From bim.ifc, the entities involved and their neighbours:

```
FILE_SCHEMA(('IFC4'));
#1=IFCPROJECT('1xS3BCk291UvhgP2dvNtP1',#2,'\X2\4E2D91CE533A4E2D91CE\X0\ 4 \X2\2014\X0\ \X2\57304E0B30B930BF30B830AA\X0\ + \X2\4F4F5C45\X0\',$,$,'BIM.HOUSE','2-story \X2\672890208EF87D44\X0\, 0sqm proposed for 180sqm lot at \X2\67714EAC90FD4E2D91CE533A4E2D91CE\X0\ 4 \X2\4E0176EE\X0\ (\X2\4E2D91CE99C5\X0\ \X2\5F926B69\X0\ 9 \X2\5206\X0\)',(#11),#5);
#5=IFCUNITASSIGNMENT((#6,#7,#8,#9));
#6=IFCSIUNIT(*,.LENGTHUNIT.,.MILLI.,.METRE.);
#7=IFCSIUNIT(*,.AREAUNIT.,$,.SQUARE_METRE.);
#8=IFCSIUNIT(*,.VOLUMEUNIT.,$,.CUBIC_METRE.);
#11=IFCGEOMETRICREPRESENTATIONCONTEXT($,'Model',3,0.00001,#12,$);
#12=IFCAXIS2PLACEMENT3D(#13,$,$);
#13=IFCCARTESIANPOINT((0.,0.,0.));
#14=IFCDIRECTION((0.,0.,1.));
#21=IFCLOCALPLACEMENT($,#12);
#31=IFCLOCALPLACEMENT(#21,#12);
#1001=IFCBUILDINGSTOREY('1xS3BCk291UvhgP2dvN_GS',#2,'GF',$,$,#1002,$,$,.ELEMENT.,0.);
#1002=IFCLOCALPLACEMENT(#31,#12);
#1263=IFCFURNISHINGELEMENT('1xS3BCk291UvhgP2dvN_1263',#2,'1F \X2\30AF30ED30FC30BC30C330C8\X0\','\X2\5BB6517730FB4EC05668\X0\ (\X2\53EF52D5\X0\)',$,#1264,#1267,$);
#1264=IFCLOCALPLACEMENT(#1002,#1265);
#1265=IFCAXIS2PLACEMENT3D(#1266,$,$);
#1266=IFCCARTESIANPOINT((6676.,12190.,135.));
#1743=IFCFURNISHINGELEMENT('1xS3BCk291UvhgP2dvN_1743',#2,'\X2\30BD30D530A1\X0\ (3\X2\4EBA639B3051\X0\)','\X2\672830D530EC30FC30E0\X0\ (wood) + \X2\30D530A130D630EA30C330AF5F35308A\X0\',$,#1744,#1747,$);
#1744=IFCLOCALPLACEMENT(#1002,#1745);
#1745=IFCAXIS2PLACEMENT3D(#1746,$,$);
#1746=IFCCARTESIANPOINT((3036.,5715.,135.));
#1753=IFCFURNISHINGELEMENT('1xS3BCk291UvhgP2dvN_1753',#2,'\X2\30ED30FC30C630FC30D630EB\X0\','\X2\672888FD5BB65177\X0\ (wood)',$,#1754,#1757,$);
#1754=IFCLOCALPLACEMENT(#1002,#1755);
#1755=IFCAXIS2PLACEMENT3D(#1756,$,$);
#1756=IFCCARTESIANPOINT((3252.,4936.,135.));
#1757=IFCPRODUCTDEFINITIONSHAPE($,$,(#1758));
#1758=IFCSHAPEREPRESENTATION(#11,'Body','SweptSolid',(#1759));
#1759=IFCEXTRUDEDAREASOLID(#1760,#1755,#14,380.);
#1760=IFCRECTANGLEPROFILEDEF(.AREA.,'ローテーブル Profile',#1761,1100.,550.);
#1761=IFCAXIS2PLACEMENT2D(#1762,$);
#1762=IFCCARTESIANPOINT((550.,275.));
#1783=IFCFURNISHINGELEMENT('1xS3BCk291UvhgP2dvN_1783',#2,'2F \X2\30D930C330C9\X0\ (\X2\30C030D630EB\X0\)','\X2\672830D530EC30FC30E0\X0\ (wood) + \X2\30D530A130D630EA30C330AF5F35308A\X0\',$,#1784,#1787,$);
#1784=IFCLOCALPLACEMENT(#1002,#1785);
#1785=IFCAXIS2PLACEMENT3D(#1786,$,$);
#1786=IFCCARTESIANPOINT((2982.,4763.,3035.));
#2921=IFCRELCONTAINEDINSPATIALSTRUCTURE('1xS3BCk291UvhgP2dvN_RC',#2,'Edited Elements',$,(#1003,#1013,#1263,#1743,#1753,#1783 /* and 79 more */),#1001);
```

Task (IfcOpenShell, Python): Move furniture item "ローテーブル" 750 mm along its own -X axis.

```python
import ifcopenshell
import ifcopenshell.api.geometry
import ifcopenshell.util.placement
import ifcopenshell.util.unit

model = ifcopenshell.open("bim.ifc")
unit_scale = ifcopenshell.util.unit.calculate_unit_scale(model)

item = model.by_guid("1xS3BCk291UvhgP2dvN_1753")
matrix = ifcopenshell.util.placement.get_local_placement(item.ObjectPlacement)
matrix[:3, 3] -= matrix[:3, 0] * 0.75 / unit_scale
ifcopenshell.api.geometry.edit_object_placement(model, product=item, matrix=matrix, is_si=False)

print(ifcopenshell.util.placement.get_local_placement(item.ObjectPlacement).round(3) + 0.0)

model.write("bim_updated.ifc")
```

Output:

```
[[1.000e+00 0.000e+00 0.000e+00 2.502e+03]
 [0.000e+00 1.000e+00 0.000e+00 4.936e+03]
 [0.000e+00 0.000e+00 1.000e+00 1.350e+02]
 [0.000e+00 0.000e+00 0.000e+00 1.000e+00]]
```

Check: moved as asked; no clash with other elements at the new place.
